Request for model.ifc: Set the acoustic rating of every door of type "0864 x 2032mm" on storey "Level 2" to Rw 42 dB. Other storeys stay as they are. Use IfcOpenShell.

First a look at what the model holds.

```python
import ifcopenshell
import ifcopenshell.util.element

model = ifcopenshell.open("model.ifc")
print(model.schema)
storey = next(s for s in model.by_type("IfcBuildingStorey") if s.Name == "Level 2")
doors = [e for e in ifcopenshell.util.element.get_decomposition(storey) if e.is_a("IfcDoor")]
seen = {}
for e in doors:
    element_type = ifcopenshell.util.element.get_type(e)
    key = (element_type.Name if element_type != e and element_type else None, ifcopenshell.util.element.get_pset(e, "Pset_DoorCommon", "AcousticRating"))
    seen[key] = seen.get(key, 0) + 1
for (name, value), count in sorted(seen.items(), key=str):
    print(count, "x", name, "|", value)
```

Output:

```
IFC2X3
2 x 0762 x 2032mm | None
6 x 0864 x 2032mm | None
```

```python
import ifcopenshell
import ifcopenshell.api.pset
import ifcopenshell.util.element

model = ifcopenshell.open("model.ifc")

storey = next(s for s in model.by_type("IfcBuildingStorey") if s.Name == "Level 2")
doors = [e for e in ifcopenshell.util.element.get_decomposition(storey) if e.is_a("IfcDoor")]

count = 0
for e in doors:
    element_type = ifcopenshell.util.element.get_type(e)
    if element_type in (None, e) or element_type.Name != "0864 x 2032mm":
        continue
    # add_pset returns the element's existing set when there is one.
    pset = ifcopenshell.api.pset.add_pset(model, product=e, name="Pset_DoorCommon")
    ifcopenshell.api.pset.edit_pset(model, pset=pset, properties={"AcousticRating": "Rw 42 dB"})
    count += 1

print(count, "doors updated")

model.write("model_updated.ifc")
```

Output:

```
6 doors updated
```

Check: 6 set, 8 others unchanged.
